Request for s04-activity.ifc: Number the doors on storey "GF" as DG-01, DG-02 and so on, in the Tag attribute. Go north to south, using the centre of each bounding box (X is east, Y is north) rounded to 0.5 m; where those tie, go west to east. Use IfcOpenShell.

First a look at what the model holds.

```python
import ifcopenshell
import ifcopenshell.util.element
import ifcopenshell.util.placement

model = ifcopenshell.open("s04-activity.ifc")
print(model.schema)
storey = next(s for s in model.by_type("IfcBuildingStorey") if s.Name == "GF")
doors = [e for e in ifcopenshell.util.element.get_decomposition(storey) if e.is_a("IfcDoor")]
for e in sorted(doors, key=lambda e: e.id()):
    origin = ifcopenshell.util.placement.get_local_placement(e.ObjectPlacement)[:3, 3]
    print(e.id(), e.Tag, e.Name, origin.round(2) + 0.0, sep=" | ")
```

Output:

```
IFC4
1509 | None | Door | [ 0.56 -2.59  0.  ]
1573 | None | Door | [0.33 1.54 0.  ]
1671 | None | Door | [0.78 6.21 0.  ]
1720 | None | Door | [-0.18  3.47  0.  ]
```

```python
import ifcopenshell
import ifcopenshell.geom
import ifcopenshell.util.element
import ifcopenshell.util.shape

model = ifcopenshell.open("s04-activity.ifc")
settings = ifcopenshell.geom.settings()
settings.set("use-world-coords", True)


def centre(element):
    shape = ifcopenshell.geom.create_shape(settings, element)
    return ifcopenshell.util.shape.get_bbox_centroid(shape.geometry)


storey = next(s for s in model.by_type("IfcBuildingStorey") if s.Name == "GF")
doors = [e for e in ifcopenshell.util.element.get_decomposition(storey) if e.is_a("IfcDoor")]

# Insertion points can sit at a corner or the storey origin, so sort by the geometry (in metres).
centres = {e: centre(e) for e in doors}
doors.sort(key=lambda e: (-round(centres[e][1] / 0.5), centres[e][0]))

for i, e in enumerate(doors, start=1):
    number = f"DG-{i:02d}"
    e.Tag = number
    print(e.id(), number)

model.write("s04-activity_v2.ifc")
```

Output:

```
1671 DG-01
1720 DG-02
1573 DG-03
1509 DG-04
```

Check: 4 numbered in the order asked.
